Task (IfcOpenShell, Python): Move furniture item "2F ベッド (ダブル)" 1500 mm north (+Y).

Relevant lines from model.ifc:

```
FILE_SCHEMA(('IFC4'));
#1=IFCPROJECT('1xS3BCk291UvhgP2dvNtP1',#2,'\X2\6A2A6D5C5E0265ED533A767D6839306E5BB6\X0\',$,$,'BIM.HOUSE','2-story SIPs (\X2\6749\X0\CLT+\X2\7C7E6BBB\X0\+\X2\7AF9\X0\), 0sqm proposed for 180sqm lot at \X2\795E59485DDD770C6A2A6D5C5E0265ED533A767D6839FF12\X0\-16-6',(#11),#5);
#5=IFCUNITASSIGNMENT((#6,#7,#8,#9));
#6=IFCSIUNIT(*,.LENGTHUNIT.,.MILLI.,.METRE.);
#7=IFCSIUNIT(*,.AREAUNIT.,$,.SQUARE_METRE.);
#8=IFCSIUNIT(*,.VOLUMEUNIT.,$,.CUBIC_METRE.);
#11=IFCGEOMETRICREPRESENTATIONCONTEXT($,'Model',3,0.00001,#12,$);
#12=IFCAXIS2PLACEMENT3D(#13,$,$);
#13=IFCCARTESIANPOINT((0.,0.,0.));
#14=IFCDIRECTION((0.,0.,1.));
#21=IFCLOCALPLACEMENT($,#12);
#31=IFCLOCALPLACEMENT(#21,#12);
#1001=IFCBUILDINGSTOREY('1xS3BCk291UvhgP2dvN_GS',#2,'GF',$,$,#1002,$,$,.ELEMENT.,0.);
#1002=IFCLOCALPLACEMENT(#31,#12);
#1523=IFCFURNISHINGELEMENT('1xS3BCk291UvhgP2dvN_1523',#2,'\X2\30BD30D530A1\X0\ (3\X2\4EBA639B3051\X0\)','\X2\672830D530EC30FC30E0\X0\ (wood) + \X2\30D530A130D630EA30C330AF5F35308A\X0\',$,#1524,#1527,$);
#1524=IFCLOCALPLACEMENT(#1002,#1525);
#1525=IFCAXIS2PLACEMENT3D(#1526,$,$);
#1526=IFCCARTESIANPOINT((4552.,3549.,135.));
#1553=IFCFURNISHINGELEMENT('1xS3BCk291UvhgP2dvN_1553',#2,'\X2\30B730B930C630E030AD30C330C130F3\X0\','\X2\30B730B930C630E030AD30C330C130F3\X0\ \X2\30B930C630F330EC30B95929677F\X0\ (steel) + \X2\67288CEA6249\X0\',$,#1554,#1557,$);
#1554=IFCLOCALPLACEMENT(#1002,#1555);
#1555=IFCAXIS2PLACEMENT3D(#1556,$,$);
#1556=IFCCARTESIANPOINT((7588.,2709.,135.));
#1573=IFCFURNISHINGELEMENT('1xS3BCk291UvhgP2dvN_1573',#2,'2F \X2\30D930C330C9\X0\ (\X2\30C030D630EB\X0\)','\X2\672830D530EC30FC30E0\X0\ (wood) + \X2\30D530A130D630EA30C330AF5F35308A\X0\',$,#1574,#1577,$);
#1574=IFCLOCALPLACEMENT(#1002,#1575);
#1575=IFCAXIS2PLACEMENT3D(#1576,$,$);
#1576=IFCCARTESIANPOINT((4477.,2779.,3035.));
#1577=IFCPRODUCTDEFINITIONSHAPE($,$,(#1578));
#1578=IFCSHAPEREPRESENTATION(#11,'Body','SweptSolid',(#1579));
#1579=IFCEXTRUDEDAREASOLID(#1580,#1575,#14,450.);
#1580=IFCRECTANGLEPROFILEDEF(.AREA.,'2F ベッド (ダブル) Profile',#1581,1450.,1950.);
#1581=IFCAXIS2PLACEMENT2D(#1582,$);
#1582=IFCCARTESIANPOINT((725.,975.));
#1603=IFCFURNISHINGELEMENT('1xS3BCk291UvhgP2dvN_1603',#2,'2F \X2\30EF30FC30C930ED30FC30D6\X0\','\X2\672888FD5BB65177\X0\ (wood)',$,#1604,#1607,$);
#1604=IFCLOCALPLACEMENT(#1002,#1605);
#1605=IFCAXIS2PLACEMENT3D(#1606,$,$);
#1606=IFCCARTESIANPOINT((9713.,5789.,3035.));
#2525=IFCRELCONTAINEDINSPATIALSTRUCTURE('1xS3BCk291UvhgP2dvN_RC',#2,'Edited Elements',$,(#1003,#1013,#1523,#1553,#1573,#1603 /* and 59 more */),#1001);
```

```python
import ifcopenshell
import ifcopenshell.api.geometry
import ifcopenshell.util.placement
import ifcopenshell.util.unit

model = ifcopenshell.open("model.ifc")
unit_scale = ifcopenshell.util.unit.calculate_unit_scale(model)

item = model.by_guid("1xS3BCk291UvhgP2dvN_1573")
matrix = ifcopenshell.util.placement.get_local_placement(item.ObjectPlacement)
matrix[1, 3] += 1.5 / unit_scale
ifcopenshell.api.geometry.edit_object_placement(model, product=item, matrix=matrix, is_si=False)

print(ifcopenshell.util.placement.get_local_placement(item.ObjectPlacement).round(3) + 0.0)

model.write("model_v2.ifc")
```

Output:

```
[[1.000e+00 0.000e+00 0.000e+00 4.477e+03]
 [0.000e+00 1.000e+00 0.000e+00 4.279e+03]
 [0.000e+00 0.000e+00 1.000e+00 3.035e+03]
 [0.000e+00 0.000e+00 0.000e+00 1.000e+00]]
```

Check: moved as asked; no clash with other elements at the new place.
